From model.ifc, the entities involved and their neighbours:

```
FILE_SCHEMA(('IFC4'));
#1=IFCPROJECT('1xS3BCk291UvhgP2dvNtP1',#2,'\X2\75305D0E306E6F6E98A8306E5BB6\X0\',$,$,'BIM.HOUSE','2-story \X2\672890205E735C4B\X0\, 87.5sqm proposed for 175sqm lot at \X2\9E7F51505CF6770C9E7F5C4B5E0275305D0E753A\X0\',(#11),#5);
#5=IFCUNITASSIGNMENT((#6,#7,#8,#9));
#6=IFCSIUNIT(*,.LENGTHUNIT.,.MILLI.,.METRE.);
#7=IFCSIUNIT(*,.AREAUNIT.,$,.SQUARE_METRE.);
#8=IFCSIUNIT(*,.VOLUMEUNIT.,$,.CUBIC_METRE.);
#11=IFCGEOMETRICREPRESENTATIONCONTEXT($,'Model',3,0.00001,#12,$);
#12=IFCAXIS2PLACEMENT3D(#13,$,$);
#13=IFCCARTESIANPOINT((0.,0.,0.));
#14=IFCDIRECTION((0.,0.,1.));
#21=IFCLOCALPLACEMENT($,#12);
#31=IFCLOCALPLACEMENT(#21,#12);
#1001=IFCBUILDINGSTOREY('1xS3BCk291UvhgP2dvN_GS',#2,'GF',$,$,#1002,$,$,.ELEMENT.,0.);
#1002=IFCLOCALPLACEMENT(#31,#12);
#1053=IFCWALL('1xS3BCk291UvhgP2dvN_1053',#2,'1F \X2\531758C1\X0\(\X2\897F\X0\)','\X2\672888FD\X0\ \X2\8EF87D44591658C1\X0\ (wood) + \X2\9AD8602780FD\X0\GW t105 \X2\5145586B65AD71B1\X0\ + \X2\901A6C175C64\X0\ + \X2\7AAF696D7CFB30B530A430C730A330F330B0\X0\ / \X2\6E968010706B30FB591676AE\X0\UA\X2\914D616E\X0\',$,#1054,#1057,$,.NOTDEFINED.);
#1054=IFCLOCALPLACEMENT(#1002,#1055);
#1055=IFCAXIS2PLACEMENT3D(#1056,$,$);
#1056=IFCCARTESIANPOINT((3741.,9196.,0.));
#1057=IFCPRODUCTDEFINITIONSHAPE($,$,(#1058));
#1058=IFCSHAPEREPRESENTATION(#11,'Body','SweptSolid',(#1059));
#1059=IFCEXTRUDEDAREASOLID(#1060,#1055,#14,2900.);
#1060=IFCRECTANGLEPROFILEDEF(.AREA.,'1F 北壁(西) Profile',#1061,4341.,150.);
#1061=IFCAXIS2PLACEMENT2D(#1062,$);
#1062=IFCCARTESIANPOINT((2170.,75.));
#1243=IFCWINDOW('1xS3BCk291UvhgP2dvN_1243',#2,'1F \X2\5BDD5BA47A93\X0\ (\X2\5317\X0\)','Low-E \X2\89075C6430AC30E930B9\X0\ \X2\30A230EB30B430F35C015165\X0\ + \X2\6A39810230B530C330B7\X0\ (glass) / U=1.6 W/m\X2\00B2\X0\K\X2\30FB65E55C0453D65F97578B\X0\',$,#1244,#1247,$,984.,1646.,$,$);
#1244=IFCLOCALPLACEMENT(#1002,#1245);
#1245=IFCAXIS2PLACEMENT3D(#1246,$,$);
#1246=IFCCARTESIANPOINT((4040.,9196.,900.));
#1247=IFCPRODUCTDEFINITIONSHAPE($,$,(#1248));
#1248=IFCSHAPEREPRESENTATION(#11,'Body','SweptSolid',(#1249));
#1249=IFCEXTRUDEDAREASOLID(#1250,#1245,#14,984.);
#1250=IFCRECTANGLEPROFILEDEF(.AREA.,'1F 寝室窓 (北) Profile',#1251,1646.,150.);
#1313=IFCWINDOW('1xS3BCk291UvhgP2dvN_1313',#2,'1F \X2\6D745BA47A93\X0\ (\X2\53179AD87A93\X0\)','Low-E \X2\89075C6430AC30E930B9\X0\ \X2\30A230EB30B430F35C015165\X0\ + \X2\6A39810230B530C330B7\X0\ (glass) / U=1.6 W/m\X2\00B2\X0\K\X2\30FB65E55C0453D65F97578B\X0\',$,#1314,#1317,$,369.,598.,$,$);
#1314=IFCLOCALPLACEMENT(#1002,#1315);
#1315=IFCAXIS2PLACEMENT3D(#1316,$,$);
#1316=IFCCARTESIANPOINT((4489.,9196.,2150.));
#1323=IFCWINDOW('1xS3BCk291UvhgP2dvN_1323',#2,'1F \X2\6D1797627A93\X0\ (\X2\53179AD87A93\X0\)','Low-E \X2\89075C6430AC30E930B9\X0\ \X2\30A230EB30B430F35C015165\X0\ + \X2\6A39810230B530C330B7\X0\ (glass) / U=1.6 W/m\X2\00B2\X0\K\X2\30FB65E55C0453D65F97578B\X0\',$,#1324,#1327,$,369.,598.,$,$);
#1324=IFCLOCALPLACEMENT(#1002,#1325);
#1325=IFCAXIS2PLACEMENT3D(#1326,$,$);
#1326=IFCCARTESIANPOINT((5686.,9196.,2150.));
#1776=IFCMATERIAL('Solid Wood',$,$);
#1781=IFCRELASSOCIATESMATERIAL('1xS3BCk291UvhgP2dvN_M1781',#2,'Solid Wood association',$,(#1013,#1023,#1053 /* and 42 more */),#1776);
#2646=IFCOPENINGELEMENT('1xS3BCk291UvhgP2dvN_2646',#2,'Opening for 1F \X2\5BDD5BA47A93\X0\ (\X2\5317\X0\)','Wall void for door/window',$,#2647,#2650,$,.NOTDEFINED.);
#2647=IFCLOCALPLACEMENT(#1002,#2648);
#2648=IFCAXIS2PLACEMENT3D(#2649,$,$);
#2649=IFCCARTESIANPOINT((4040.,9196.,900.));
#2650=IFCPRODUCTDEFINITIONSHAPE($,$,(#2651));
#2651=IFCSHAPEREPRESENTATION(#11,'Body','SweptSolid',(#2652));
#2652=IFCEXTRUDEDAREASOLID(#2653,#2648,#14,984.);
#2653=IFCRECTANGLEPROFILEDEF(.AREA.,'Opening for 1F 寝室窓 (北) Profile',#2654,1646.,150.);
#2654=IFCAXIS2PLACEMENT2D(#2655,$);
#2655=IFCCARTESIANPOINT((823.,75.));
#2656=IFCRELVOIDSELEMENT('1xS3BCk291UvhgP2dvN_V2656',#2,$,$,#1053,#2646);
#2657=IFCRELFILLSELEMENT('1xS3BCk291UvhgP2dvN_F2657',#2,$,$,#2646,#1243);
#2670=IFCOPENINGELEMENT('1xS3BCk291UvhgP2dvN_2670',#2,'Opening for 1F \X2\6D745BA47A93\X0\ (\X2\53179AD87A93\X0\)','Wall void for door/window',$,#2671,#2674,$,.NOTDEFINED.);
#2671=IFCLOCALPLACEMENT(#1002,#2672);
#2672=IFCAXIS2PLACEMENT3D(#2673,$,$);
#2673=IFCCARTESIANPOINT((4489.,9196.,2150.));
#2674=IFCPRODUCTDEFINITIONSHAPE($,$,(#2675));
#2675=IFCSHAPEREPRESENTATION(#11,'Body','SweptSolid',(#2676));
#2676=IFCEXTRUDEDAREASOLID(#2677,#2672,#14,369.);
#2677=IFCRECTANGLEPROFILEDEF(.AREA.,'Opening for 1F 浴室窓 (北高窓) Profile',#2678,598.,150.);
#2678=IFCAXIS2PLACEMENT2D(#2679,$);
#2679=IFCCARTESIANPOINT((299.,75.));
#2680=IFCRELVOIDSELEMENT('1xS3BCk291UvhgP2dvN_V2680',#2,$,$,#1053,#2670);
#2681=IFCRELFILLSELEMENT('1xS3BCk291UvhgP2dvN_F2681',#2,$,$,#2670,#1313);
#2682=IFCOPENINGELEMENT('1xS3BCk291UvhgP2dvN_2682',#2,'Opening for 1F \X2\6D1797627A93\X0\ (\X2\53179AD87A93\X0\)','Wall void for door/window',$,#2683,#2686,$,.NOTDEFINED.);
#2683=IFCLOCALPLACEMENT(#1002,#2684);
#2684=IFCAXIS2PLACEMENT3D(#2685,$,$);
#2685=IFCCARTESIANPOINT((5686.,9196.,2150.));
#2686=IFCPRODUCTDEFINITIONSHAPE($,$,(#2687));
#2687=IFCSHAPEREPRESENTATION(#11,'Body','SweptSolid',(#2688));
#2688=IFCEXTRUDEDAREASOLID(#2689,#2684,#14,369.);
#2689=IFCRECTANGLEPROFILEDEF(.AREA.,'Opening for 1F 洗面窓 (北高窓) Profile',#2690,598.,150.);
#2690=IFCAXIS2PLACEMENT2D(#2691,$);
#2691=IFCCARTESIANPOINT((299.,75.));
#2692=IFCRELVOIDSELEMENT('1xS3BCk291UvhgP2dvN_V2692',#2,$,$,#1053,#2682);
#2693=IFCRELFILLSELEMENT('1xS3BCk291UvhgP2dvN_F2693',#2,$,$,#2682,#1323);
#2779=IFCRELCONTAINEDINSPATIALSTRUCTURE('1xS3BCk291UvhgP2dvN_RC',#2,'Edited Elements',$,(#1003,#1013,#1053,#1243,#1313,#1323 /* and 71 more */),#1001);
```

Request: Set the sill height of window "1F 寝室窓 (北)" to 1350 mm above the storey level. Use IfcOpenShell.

```python
import numpy as np
import ifcopenshell
import ifcopenshell.api.geometry
import ifcopenshell.geom
import ifcopenshell.util.element
import ifcopenshell.util.placement
import ifcopenshell.util.shape
import ifcopenshell.util.unit

model = ifcopenshell.open("model.ifc")
unit_scale = ifcopenshell.util.unit.calculate_unit_scale(model)

window = model.by_guid("1xS3BCk291UvhgP2dvN_1243")
opening = window.FillsVoids[0].RelatingOpeningElement
storey = ifcopenshell.util.element.get_container(window, ifc_class="IfcBuildingStorey")
level = ifcopenshell.util.placement.get_local_placement(storey.ObjectPlacement)[2, 3]

# The opening's origin need not be at the sill, so measure its lowest point.
shape = ifcopenshell.geom.create_shape(ifcopenshell.geom.settings(), opening)
bottom = ifcopenshell.util.shape.get_shape_bottom_elevation(shape, shape.geometry) / unit_scale
dz = level + 1350.0 - bottom

shift = np.array([0.0, 0.0, dz])
# The window is not placed relative to its opening, so move both.
for product in (opening, window):
    matrix = ifcopenshell.util.placement.get_local_placement(product.ObjectPlacement)
    matrix[:3, 3] += shift
    ifcopenshell.api.geometry.edit_object_placement(model, product=product, matrix=matrix, is_si=False)

print(f"moved by {dz * unit_scale:+.3f} m")

model.write("model-out.ifc")
```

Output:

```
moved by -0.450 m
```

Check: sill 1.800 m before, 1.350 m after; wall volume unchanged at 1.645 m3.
